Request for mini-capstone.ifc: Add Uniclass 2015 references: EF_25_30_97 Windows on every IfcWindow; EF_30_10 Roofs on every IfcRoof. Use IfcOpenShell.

First a look at what the model holds.

```python
import ifcopenshell

model = ifcopenshell.open("mini-capstone.ifc")
print(model.schema)
print("classifications:", [c.Name for c in model.by_type("IfcClassification")])
for ifc_class in ("IfcDoor", "IfcRoof", "IfcStair", "IfcWall", "IfcWindow"):
    print(ifc_class, len(model.by_type(ifc_class)))
```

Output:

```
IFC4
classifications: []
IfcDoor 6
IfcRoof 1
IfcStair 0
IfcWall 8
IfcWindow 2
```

```python
import ifcopenshell
import ifcopenshell.api.classification

model = ifcopenshell.open("mini-capstone.ifc")

system = ifcopenshell.api.classification.add_classification(model, classification="Uniclass 2015")

codes = {
    "IfcWindow": ("EF_25_30_97", "Windows"),
    "IfcRoof": ("EF_30_10", "Roofs"),
}
for ifc_class, (code, name) in codes.items():
    products = model.by_type(ifc_class)
    ifcopenshell.api.classification.add_reference(
        model, products=products, classification=system, identification=code, name=name
    )
    print(code, len(products))

model.write("mini-capstone_edited.ifc")
```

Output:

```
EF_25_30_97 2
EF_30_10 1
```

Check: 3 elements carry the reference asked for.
